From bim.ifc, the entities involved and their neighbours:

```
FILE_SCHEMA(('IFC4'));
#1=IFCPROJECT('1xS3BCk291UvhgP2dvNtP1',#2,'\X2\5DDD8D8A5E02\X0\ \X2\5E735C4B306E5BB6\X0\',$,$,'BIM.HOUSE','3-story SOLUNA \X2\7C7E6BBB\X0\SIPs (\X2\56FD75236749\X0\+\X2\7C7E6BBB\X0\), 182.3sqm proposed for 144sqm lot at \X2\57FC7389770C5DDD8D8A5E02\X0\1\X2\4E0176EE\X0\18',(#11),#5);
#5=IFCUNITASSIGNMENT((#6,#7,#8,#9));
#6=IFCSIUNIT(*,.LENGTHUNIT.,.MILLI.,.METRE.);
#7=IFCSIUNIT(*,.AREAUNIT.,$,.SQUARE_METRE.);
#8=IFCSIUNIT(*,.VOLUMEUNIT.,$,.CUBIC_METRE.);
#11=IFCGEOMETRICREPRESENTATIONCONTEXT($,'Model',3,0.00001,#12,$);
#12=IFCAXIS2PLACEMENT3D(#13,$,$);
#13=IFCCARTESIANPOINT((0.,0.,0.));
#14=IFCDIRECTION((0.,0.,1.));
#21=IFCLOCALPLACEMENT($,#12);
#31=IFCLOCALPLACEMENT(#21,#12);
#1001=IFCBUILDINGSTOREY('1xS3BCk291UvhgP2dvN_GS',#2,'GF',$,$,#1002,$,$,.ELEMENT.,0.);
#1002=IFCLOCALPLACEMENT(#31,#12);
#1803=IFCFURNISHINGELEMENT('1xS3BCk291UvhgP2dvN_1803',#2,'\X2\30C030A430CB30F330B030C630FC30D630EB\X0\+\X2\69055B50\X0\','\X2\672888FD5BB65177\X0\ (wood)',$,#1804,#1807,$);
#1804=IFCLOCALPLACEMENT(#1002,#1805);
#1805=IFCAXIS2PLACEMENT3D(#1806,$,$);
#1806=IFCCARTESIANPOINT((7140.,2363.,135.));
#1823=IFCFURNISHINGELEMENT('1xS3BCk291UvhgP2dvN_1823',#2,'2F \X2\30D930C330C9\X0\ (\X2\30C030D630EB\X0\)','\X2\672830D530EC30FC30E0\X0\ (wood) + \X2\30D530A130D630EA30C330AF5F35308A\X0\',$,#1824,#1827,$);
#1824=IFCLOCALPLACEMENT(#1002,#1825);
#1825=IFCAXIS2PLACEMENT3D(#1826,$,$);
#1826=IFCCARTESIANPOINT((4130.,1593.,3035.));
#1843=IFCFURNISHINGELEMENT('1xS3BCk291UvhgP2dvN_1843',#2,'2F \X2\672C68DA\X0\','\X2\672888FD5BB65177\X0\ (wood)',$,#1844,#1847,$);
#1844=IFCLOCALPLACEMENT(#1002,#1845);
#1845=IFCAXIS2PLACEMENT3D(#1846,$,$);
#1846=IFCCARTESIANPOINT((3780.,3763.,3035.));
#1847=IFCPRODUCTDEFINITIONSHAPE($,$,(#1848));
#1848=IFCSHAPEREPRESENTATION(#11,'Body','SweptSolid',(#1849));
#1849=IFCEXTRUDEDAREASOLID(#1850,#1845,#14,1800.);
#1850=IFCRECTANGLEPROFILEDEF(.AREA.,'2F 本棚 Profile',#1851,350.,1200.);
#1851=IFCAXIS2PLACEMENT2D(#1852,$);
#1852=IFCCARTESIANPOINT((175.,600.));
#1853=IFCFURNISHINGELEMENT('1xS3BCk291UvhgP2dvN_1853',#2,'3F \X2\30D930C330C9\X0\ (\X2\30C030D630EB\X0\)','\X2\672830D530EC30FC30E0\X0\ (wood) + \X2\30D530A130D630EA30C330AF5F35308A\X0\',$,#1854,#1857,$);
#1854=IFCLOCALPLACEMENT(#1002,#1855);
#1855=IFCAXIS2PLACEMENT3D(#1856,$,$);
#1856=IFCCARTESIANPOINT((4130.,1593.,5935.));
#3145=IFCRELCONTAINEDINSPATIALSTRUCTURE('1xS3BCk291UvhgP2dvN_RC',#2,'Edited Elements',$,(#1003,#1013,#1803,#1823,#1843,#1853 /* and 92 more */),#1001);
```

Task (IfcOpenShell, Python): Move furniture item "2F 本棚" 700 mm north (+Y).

```python
import ifcopenshell
import ifcopenshell.api.geometry
import ifcopenshell.util.placement
import ifcopenshell.util.unit

model = ifcopenshell.open("bim.ifc")
unit_scale = ifcopenshell.util.unit.calculate_unit_scale(model)

item = model.by_guid("1xS3BCk291UvhgP2dvN_1843")
matrix = ifcopenshell.util.placement.get_local_placement(item.ObjectPlacement)
matrix[1, 3] += 0.7 / unit_scale
ifcopenshell.api.geometry.edit_object_placement(model, product=item, matrix=matrix, is_si=False)

print(ifcopenshell.util.placement.get_local_placement(item.ObjectPlacement).round(3) + 0.0)

model.write("bim_updated.ifc")
```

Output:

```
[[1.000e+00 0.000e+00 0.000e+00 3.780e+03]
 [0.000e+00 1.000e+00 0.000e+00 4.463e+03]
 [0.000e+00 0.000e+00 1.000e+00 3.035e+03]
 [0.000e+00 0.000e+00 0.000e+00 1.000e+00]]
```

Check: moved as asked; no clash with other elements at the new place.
